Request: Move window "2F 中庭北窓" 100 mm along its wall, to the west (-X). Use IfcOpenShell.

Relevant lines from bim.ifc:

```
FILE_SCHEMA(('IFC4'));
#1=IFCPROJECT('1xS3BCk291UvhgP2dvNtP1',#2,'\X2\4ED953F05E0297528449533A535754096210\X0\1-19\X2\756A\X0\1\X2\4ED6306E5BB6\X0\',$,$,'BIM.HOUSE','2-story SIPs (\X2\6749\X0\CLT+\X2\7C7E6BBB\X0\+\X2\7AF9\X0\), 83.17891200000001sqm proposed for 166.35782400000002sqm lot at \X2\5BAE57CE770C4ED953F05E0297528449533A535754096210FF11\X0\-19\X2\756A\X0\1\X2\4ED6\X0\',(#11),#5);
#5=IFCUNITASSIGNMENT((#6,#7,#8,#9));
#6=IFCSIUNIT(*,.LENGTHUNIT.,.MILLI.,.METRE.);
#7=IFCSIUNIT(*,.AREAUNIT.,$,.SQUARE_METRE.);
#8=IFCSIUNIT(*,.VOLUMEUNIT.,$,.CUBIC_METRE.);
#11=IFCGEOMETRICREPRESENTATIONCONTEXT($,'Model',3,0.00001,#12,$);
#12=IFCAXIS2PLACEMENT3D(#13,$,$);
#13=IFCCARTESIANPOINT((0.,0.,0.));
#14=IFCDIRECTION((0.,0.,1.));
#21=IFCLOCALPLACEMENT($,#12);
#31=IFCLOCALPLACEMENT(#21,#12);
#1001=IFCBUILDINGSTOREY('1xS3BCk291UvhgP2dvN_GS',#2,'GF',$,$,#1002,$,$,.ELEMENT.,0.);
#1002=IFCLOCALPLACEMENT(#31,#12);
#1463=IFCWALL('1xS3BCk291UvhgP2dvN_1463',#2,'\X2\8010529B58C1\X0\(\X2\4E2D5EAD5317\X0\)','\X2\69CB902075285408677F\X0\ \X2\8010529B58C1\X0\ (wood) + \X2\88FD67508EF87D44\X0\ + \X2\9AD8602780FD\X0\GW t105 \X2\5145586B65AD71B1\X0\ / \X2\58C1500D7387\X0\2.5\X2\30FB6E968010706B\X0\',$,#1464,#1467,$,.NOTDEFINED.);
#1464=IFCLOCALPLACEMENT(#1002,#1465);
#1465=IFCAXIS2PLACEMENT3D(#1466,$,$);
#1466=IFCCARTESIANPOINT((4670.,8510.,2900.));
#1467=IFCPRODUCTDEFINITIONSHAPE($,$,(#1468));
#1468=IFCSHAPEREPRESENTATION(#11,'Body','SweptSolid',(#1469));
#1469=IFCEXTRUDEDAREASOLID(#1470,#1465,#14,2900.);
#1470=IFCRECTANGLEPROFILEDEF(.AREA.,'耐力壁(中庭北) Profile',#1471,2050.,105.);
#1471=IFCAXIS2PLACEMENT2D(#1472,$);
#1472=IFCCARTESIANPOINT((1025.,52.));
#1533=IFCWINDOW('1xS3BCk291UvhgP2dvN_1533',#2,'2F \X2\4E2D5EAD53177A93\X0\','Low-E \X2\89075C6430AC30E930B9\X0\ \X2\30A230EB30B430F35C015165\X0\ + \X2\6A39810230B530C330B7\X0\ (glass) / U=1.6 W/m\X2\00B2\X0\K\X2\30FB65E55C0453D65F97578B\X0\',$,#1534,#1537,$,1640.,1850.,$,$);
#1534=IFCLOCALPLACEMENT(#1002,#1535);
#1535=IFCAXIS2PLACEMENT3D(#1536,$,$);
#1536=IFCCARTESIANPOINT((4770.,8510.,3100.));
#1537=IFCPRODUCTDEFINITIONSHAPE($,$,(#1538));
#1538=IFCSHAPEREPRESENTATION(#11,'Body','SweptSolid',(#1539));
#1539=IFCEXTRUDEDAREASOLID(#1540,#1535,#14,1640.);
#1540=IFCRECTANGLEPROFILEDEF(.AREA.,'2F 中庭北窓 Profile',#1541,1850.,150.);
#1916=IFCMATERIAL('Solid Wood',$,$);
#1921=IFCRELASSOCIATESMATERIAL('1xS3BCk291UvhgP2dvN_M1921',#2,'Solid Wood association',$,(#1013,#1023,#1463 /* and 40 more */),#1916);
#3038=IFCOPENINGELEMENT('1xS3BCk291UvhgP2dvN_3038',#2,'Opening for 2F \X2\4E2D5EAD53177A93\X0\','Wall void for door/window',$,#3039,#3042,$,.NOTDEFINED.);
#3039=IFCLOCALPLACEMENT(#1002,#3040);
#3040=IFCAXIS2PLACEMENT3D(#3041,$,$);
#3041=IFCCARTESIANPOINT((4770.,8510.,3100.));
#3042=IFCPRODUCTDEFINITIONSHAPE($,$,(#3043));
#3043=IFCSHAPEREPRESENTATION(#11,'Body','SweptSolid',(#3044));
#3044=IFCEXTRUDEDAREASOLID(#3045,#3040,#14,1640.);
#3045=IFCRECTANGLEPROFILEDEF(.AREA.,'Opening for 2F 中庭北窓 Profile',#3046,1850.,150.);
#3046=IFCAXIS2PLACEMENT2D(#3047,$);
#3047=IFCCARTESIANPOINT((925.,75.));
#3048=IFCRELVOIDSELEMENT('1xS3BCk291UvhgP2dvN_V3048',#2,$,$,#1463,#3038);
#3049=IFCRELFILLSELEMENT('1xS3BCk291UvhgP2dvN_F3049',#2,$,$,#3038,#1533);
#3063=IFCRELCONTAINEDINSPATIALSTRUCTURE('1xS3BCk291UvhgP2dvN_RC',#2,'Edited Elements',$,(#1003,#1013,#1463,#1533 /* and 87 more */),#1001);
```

```python
import ifcopenshell
import ifcopenshell.api.geometry
import ifcopenshell.util.placement
import ifcopenshell.util.unit

model = ifcopenshell.open("bim.ifc")
unit_scale = ifcopenshell.util.unit.calculate_unit_scale(model)

window = model.by_guid("1xS3BCk291UvhgP2dvN_1533")
opening = window.FillsVoids[0].RelatingOpeningElement
wall = opening.VoidsElements[0].RelatingBuildingElement

wall_matrix = ifcopenshell.util.placement.get_local_placement(wall.ObjectPlacement)
shift = wall_matrix[:3, 0] * -0.1 / unit_scale
before = ifcopenshell.util.placement.get_local_placement(window.ObjectPlacement)[:3, 3].copy()

# The window is not placed relative to its opening, so move both.
for product in (opening, window):
    matrix = ifcopenshell.util.placement.get_local_placement(product.ObjectPlacement)
    matrix[:3, 3] += shift
    ifcopenshell.api.geometry.edit_object_placement(model, product=product, matrix=matrix, is_si=False)

after = ifcopenshell.util.placement.get_local_placement(window.ObjectPlacement)[:3, 3]
print("window moved by", (after - before).round(3) + 0.0)

model.write("bim_edited.ifc")
```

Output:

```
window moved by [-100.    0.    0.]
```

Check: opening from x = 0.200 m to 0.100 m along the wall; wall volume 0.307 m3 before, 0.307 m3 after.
